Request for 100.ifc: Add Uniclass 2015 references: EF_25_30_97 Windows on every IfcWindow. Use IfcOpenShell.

First a look at what the model holds.

```python
import ifcopenshell

model = ifcopenshell.open("100.ifc")
print(model.schema)
print("classifications:", [c.Name for c in model.by_type("IfcClassification")])
for ifc_class in ("IfcDoor", "IfcRoof", "IfcStair", "IfcWall", "IfcWindow"):
    print(ifc_class, len(model.by_type(ifc_class)))
```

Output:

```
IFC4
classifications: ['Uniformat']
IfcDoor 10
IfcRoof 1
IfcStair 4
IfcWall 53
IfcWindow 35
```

```python
import ifcopenshell
import ifcopenshell.api.classification

model = ifcopenshell.open("100.ifc")

system = ifcopenshell.api.classification.add_classification(model, classification="Uniclass 2015")

codes = {
    "IfcWindow": ("EF_25_30_97", "Windows"),
}
for ifc_class, (code, name) in codes.items():
    products = model.by_type(ifc_class)
    ifcopenshell.api.classification.add_reference(
        model, products=products, classification=system, identification=code, name=name
    )
    print(code, len(products))

model.write("100-out.ifc")
```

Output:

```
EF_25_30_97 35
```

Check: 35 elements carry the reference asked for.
